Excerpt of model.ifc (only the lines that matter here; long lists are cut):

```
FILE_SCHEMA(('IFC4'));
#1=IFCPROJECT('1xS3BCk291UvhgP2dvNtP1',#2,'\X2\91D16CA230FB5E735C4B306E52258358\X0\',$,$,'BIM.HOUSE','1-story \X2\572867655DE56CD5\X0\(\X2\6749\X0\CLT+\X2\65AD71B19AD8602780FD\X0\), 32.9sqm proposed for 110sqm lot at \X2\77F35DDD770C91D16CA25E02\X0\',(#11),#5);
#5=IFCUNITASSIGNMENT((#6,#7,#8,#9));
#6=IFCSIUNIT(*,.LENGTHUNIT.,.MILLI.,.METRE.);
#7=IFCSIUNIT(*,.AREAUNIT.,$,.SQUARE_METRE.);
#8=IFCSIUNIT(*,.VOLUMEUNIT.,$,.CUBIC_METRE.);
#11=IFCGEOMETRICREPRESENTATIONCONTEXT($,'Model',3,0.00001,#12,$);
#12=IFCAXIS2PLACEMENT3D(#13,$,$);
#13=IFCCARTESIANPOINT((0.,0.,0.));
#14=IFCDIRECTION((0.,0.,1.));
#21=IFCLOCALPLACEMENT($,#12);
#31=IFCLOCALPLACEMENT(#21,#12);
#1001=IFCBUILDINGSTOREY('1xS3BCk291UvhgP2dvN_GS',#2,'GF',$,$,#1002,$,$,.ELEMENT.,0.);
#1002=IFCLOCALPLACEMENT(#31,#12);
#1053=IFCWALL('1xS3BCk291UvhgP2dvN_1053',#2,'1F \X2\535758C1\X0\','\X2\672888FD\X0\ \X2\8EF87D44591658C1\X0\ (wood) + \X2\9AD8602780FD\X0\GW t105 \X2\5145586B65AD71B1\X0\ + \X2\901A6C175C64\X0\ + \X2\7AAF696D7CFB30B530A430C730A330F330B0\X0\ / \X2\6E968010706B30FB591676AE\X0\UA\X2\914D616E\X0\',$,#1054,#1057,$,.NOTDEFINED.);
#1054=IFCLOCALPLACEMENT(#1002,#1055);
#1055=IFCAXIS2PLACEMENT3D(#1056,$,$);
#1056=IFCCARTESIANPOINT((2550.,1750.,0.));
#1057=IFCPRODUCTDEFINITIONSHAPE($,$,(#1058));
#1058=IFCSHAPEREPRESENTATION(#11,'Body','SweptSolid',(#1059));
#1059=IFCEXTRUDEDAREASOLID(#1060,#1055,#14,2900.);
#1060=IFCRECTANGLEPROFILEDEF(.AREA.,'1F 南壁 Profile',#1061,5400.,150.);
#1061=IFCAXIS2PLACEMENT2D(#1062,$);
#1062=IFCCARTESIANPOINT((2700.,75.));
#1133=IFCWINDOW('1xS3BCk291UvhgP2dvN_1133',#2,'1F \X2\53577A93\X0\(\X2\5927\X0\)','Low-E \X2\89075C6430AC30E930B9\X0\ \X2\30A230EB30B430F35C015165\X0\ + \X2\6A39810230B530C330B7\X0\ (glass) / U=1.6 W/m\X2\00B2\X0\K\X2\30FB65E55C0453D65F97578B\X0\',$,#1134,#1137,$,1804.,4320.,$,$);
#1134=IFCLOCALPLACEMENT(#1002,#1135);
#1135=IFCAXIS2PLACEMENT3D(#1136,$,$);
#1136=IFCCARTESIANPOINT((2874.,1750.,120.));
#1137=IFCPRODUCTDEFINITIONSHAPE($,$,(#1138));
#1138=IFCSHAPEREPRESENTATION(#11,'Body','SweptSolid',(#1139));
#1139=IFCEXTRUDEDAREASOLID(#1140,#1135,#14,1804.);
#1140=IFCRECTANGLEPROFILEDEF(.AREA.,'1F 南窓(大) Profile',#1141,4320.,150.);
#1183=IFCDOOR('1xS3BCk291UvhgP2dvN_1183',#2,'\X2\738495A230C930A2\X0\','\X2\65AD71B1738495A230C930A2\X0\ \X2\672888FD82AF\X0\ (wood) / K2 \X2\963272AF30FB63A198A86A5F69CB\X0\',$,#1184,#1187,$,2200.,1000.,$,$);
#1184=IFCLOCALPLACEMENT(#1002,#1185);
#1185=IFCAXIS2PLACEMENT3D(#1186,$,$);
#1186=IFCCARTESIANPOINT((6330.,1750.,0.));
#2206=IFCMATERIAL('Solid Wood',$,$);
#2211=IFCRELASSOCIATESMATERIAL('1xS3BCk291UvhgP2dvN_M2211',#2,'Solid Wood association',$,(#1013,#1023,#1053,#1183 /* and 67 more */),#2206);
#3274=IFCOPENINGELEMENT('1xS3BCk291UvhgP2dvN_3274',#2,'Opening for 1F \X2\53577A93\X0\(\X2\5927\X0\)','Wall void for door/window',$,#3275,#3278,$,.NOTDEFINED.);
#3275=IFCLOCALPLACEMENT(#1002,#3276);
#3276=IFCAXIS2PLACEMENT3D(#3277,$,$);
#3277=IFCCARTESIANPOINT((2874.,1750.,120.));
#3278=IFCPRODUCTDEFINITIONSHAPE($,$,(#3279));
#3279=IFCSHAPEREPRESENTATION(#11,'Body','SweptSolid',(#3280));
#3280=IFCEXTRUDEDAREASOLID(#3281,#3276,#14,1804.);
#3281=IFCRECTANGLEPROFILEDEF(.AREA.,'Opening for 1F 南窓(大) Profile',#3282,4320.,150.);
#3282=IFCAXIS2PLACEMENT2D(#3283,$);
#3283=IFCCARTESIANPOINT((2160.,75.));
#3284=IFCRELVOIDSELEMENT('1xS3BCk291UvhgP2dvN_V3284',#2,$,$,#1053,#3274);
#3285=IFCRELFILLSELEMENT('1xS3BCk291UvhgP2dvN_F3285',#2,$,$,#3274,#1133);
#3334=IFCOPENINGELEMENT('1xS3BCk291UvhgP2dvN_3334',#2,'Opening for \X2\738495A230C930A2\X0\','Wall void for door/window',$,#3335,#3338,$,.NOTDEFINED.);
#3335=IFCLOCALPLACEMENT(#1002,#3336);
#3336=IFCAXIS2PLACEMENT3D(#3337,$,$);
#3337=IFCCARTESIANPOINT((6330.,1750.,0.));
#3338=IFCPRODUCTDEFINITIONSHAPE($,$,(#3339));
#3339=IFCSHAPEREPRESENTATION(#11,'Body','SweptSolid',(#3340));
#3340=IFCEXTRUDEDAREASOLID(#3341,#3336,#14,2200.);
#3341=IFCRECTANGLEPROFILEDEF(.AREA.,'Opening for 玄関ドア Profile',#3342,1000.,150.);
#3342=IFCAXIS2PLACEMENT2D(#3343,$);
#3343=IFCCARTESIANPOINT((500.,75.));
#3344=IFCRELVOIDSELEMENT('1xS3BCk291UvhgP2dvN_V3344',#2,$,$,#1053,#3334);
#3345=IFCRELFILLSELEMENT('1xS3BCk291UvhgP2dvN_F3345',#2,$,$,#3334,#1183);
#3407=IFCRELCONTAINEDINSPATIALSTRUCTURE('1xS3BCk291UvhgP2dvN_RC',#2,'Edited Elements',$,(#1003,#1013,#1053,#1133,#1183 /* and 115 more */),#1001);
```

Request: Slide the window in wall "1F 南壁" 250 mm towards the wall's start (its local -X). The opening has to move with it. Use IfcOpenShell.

```python
import ifcopenshell
import ifcopenshell.api.geometry
import ifcopenshell.util.placement

model = ifcopenshell.open("model.ifc")

window = model.by_guid("1xS3BCk291UvhgP2dvN_1133")
opening = window.FillsVoids[0].RelatingOpeningElement
wall = opening.VoidsElements[0].RelatingBuildingElement

wall_matrix = ifcopenshell.util.placement.get_local_placement(wall.ObjectPlacement)
shift = wall_matrix[:3, 0] * -250.0
before = ifcopenshell.util.placement.get_local_placement(window.ObjectPlacement)[:3, 3].copy()

# The window is not placed relative to its opening, so move both.
for product in (opening, window):
    matrix = ifcopenshell.util.placement.get_local_placement(product.ObjectPlacement)
    matrix[:3, 3] += shift
    ifcopenshell.api.geometry.edit_object_placement(model, product=product, matrix=matrix, is_si=False)

after = ifcopenshell.util.placement.get_local_placement(window.ObjectPlacement)[:3, 3]
print("window moved by", (after - before).round(3) + 0.0)

model.write("model_updated.ifc")
```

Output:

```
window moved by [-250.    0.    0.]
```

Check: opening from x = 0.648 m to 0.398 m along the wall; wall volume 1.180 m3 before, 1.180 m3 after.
